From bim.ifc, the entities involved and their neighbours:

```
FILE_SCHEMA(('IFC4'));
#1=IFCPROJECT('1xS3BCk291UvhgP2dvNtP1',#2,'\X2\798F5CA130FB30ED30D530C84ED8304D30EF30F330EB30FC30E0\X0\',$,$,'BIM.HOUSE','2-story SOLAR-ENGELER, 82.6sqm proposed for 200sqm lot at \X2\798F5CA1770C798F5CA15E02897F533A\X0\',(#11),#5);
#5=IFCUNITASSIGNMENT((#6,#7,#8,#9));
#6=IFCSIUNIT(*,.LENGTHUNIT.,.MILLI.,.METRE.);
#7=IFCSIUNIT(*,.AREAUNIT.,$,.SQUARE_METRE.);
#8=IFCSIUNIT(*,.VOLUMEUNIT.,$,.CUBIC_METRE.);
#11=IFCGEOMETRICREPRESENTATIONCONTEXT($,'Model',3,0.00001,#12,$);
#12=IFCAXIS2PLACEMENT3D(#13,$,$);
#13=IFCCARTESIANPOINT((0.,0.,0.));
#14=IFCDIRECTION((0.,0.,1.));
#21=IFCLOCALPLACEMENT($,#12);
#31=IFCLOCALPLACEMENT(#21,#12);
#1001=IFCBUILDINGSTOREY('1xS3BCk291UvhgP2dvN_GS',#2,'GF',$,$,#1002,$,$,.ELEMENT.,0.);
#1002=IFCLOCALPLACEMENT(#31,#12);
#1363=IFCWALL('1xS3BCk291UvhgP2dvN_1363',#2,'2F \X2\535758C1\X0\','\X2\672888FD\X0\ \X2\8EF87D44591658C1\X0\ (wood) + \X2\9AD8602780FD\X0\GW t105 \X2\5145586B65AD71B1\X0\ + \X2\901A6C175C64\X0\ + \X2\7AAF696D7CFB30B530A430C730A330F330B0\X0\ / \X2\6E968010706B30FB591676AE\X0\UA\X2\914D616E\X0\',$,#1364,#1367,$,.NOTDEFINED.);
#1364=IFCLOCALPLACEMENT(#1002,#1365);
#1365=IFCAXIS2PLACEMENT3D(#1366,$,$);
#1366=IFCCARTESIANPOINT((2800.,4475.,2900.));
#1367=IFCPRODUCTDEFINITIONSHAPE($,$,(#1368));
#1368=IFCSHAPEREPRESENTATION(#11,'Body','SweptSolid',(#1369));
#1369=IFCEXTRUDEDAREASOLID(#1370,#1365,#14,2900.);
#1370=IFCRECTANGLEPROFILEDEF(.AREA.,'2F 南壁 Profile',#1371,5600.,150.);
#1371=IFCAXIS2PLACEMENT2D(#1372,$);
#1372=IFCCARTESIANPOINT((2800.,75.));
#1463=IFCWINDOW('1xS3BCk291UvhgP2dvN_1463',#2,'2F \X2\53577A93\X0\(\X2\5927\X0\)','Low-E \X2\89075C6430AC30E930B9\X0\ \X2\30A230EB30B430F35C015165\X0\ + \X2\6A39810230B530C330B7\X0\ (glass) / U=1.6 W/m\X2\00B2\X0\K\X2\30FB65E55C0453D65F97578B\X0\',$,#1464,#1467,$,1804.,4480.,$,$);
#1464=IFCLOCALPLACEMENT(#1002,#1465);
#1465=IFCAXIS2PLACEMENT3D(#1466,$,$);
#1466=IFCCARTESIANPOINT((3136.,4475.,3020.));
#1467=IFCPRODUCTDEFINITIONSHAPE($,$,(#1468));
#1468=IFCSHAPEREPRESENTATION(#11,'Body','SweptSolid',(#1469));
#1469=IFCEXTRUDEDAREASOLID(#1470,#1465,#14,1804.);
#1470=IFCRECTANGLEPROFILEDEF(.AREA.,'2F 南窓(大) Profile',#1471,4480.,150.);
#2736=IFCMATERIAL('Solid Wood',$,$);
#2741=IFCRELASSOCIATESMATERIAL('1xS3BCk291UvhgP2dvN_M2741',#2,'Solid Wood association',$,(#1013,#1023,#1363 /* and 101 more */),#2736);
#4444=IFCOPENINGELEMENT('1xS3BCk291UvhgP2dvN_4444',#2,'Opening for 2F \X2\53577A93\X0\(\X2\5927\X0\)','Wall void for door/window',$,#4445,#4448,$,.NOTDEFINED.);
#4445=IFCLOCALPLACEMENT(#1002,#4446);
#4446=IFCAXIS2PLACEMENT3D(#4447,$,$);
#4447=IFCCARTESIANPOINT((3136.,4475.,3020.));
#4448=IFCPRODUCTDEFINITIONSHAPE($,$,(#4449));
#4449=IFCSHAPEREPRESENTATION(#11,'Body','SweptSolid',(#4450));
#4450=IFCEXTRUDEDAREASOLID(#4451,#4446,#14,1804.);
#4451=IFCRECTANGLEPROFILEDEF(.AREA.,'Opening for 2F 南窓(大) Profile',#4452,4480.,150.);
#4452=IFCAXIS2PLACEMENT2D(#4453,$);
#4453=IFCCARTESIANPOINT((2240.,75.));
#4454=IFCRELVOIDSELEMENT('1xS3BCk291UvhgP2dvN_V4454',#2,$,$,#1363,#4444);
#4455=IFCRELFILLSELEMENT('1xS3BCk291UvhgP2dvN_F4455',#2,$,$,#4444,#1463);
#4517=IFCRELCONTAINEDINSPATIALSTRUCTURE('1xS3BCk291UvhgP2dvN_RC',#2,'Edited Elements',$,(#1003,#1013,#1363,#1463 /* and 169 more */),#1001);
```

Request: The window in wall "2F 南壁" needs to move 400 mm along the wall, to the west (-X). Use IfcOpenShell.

```python
import ifcopenshell
import ifcopenshell.api.geometry
import ifcopenshell.util.placement
import ifcopenshell.util.unit

model = ifcopenshell.open("bim.ifc")
unit_scale = ifcopenshell.util.unit.calculate_unit_scale(model)

window = model.by_id(1463)
opening = window.FillsVoids[0].RelatingOpeningElement
wall = opening.VoidsElements[0].RelatingBuildingElement

wall_matrix = ifcopenshell.util.placement.get_local_placement(wall.ObjectPlacement)
shift = wall_matrix[:3, 0] * -0.4 / unit_scale
before = ifcopenshell.util.placement.get_local_placement(window.ObjectPlacement)[:3, 3].copy()

# The window is not placed relative to its opening, so move both.
for product in (opening, window):
    matrix = ifcopenshell.util.placement.get_local_placement(product.ObjectPlacement)
    matrix[:3, 3] += shift
    ifcopenshell.api.geometry.edit_object_placement(model, product=product, matrix=matrix, is_si=False)

after = ifcopenshell.util.placement.get_local_placement(window.ObjectPlacement)[:3, 3]
print("window moved by", (after - before).round(3) + 0.0)

model.write("bim-out.ifc")
```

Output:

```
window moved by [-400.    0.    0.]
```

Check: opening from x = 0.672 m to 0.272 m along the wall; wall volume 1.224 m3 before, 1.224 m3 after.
